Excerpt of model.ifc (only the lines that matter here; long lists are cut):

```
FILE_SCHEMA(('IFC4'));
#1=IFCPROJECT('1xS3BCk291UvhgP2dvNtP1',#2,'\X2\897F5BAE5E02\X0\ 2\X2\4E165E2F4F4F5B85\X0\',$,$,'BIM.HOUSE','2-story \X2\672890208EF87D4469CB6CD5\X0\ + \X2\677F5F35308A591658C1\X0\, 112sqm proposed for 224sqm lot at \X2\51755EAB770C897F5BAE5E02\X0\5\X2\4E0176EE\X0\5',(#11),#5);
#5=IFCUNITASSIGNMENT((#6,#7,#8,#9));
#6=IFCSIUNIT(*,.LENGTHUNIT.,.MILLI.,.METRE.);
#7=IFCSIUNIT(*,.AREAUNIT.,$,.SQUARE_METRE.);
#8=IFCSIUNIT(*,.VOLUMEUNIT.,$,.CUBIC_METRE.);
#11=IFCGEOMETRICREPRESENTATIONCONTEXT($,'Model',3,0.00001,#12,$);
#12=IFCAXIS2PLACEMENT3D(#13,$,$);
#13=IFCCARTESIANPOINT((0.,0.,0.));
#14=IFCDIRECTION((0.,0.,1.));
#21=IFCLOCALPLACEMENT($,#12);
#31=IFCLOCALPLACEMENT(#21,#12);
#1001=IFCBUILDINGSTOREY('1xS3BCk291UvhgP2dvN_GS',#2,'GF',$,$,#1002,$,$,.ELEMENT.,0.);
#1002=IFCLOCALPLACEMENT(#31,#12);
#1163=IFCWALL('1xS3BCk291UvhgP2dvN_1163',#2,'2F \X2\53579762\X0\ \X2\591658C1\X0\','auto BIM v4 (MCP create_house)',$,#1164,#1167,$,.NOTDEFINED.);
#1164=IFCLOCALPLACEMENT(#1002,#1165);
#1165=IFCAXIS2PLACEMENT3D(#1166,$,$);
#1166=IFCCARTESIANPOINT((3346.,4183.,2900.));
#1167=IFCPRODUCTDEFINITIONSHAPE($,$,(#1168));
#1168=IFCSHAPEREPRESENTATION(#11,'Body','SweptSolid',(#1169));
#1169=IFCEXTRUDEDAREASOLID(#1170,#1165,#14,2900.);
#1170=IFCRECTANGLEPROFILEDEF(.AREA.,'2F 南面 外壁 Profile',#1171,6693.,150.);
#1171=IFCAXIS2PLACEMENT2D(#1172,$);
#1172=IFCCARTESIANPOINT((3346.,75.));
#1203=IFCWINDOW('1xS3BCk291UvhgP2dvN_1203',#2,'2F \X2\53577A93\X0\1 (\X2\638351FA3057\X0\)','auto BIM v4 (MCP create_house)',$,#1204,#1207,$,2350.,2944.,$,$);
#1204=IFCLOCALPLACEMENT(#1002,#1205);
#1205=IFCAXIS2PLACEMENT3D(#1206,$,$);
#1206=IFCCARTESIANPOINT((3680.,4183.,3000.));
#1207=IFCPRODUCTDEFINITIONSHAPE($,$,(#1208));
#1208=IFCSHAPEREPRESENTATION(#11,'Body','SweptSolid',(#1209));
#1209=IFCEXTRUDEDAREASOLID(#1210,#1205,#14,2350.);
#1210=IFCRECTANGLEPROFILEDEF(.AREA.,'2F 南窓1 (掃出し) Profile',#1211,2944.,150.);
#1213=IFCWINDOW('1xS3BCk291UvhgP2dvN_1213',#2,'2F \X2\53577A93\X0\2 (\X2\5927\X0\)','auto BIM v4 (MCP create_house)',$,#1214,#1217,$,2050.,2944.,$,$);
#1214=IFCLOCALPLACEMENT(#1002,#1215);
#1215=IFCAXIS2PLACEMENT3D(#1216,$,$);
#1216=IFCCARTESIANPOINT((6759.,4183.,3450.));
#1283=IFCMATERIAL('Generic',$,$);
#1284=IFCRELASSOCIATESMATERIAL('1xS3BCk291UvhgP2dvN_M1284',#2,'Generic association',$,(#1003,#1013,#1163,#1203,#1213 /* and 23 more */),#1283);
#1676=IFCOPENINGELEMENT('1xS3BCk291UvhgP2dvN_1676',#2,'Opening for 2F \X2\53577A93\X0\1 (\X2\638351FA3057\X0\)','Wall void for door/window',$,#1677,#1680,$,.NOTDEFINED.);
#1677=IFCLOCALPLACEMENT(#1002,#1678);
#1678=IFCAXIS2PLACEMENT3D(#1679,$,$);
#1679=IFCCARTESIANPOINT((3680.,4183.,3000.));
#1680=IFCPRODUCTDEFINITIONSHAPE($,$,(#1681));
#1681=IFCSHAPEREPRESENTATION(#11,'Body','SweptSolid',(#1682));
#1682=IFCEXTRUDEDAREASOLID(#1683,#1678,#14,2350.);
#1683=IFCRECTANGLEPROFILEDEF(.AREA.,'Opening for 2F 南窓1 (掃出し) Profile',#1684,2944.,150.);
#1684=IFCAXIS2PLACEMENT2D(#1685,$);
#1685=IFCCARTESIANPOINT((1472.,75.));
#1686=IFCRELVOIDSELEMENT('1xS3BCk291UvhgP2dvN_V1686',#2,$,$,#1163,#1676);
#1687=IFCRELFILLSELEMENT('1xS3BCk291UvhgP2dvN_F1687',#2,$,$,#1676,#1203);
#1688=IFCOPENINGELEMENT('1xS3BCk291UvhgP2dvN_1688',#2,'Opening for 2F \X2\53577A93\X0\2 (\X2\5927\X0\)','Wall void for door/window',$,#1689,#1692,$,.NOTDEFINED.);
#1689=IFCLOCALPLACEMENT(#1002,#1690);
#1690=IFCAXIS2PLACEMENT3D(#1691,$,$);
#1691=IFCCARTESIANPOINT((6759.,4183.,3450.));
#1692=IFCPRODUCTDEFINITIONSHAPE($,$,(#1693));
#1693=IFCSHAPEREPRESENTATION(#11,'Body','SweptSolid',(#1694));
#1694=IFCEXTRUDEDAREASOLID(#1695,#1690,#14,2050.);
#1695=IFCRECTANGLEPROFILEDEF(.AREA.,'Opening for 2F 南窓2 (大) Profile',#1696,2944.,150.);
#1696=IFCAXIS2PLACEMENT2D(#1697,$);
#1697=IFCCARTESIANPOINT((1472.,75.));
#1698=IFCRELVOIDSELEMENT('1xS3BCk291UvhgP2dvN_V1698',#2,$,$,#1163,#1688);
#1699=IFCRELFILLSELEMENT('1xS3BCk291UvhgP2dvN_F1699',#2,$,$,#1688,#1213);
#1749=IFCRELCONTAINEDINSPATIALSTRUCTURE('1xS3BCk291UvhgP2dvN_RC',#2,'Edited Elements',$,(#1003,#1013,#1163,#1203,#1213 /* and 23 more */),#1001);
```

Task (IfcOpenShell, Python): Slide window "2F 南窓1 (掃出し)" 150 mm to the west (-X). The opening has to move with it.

```python
import ifcopenshell
import ifcopenshell.api.geometry
import ifcopenshell.util.placement
import ifcopenshell.util.unit

model = ifcopenshell.open("model.ifc")
unit_scale = ifcopenshell.util.unit.calculate_unit_scale(model)

window = model.by_guid("1xS3BCk291UvhgP2dvN_1203")
opening = window.FillsVoids[0].RelatingOpeningElement
wall = opening.VoidsElements[0].RelatingBuildingElement

wall_matrix = ifcopenshell.util.placement.get_local_placement(wall.ObjectPlacement)
shift = wall_matrix[:3, 0] * -0.15 / unit_scale
before = ifcopenshell.util.placement.get_local_placement(window.ObjectPlacement)[:3, 3].copy()

# The window is not placed relative to its opening, so move both.
for product in (opening, window):
    matrix = ifcopenshell.util.placement.get_local_placement(product.ObjectPlacement)
    matrix[:3, 3] += shift
    ifcopenshell.api.geometry.edit_object_placement(model, product=product, matrix=matrix, is_si=False)

after = ifcopenshell.util.placement.get_local_placement(window.ObjectPlacement)[:3, 3]
print("window moved by", (after - before).round(3) + 0.0)

model.write("model_edited.ifc")
```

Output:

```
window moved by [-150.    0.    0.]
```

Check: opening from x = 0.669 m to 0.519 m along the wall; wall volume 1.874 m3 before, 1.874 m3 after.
